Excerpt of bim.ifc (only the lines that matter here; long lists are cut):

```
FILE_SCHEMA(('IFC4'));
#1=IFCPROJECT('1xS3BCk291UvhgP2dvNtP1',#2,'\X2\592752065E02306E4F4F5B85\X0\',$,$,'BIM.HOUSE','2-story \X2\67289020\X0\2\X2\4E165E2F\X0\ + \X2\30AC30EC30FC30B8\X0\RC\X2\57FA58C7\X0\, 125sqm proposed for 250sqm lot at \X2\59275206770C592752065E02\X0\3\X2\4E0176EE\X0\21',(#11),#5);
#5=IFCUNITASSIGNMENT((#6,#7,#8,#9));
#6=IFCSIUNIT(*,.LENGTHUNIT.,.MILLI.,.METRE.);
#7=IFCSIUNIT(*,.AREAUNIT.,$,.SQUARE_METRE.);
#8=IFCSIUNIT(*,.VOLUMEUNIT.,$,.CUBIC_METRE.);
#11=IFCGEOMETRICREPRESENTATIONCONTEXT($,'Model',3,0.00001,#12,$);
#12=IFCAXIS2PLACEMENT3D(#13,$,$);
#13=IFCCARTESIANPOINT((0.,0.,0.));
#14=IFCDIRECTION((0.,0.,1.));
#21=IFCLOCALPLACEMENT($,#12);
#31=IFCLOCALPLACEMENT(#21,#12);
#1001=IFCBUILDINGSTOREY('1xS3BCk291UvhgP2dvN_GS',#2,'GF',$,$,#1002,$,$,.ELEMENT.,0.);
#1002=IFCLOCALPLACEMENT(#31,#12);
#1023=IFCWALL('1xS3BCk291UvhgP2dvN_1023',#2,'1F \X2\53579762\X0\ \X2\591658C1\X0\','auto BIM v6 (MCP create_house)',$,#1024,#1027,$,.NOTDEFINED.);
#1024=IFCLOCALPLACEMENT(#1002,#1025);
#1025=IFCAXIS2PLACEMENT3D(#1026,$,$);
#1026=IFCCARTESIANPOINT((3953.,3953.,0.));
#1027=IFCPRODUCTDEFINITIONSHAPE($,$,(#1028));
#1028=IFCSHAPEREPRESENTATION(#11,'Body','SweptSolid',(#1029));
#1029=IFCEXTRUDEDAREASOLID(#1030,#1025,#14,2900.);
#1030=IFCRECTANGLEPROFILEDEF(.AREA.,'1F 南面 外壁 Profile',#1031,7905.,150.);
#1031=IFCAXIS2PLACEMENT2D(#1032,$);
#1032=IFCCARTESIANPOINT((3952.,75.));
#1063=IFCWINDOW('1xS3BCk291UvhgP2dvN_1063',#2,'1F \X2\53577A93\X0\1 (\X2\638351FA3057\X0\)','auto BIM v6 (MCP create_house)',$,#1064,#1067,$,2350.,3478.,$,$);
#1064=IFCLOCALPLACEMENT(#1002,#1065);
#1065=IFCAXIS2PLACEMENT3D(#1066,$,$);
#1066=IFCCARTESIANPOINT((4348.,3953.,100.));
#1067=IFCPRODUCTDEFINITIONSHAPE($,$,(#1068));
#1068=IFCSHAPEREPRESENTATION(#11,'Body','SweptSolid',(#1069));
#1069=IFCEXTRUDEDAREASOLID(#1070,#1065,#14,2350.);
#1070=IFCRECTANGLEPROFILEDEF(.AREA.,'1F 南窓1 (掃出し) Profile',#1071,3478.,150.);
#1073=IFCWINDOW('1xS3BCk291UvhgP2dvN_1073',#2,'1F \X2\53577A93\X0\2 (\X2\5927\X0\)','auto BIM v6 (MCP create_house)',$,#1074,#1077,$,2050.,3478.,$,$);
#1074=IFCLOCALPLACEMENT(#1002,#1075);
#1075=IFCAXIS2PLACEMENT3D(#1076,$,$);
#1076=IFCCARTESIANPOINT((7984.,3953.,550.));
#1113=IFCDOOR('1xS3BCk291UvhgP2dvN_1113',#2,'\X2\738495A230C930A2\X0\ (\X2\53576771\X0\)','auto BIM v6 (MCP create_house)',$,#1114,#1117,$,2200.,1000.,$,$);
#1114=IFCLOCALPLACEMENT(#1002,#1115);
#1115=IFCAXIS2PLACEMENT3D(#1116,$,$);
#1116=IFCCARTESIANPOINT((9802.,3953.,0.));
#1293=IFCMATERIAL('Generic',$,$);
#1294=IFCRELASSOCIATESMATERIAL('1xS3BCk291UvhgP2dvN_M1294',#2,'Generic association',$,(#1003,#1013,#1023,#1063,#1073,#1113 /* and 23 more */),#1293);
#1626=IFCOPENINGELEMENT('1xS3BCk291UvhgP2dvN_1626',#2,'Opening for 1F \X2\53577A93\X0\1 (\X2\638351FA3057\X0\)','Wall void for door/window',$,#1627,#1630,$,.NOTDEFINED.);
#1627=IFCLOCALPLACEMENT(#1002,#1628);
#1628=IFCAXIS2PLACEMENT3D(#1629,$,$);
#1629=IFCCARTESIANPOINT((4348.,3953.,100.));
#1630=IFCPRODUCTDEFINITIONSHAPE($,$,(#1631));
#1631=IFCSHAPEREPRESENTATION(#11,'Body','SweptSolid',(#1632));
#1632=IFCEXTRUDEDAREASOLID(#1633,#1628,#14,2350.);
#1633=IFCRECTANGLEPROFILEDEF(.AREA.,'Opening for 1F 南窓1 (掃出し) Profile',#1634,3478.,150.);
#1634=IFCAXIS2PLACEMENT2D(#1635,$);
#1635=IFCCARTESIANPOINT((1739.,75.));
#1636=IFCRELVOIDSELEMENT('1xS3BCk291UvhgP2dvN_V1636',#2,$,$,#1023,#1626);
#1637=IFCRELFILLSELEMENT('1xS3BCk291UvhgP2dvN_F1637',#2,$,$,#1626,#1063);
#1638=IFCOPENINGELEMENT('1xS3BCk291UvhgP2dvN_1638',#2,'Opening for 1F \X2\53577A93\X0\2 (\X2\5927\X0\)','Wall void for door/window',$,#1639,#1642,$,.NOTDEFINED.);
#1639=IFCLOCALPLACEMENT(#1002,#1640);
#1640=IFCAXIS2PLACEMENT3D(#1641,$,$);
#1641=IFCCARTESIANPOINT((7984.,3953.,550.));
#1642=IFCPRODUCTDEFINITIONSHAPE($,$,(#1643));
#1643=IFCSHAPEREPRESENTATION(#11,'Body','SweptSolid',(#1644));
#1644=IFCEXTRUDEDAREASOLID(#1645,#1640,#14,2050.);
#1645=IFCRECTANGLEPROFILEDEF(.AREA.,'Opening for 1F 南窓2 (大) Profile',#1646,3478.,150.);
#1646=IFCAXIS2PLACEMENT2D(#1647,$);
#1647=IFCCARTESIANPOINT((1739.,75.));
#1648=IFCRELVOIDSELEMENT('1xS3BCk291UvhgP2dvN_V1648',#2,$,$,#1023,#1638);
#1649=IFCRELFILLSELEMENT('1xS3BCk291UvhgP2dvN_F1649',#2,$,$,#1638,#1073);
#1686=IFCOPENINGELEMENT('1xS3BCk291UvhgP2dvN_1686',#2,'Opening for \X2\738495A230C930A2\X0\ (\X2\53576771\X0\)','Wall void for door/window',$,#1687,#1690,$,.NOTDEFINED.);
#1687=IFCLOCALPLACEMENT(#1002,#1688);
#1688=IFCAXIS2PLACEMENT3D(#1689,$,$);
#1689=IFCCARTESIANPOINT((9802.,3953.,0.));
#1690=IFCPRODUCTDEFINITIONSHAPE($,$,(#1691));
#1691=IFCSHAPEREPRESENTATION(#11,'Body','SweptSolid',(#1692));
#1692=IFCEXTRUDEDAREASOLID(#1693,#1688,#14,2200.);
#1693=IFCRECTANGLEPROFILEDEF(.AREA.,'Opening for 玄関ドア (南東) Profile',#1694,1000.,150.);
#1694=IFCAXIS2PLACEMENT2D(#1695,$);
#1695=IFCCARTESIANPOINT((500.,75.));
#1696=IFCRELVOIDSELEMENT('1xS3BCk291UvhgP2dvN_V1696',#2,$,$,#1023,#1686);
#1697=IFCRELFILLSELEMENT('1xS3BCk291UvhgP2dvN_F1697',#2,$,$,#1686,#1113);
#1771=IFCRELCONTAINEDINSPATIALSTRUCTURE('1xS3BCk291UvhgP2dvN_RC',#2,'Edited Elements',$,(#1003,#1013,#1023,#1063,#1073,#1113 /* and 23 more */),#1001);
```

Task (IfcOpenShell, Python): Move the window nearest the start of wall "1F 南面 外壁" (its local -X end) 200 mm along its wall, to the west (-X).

```python
import ifcopenshell
import ifcopenshell.api.geometry
import ifcopenshell.util.placement

model = ifcopenshell.open("bim.ifc")

window = model.by_guid("1xS3BCk291UvhgP2dvN_1063")
opening = window.FillsVoids[0].RelatingOpeningElement
wall = opening.VoidsElements[0].RelatingBuildingElement

wall_matrix = ifcopenshell.util.placement.get_local_placement(wall.ObjectPlacement)
shift = wall_matrix[:3, 0] * -200.0
before = ifcopenshell.util.placement.get_local_placement(window.ObjectPlacement)[:3, 3].copy()

# The window is not placed relative to its opening, so move both.
for product in (opening, window):
    matrix = ifcopenshell.util.placement.get_local_placement(product.ObjectPlacement)
    matrix[:3, 3] += shift
    ifcopenshell.api.geometry.edit_object_placement(model, product=product, matrix=matrix, is_si=False)

after = ifcopenshell.util.placement.get_local_placement(window.ObjectPlacement)[:3, 3]
print("window moved by", (after - before).round(3) + 0.0)

model.write("bim_updated.ifc")
```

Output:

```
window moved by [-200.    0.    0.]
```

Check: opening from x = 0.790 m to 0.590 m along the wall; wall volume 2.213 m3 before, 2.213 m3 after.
